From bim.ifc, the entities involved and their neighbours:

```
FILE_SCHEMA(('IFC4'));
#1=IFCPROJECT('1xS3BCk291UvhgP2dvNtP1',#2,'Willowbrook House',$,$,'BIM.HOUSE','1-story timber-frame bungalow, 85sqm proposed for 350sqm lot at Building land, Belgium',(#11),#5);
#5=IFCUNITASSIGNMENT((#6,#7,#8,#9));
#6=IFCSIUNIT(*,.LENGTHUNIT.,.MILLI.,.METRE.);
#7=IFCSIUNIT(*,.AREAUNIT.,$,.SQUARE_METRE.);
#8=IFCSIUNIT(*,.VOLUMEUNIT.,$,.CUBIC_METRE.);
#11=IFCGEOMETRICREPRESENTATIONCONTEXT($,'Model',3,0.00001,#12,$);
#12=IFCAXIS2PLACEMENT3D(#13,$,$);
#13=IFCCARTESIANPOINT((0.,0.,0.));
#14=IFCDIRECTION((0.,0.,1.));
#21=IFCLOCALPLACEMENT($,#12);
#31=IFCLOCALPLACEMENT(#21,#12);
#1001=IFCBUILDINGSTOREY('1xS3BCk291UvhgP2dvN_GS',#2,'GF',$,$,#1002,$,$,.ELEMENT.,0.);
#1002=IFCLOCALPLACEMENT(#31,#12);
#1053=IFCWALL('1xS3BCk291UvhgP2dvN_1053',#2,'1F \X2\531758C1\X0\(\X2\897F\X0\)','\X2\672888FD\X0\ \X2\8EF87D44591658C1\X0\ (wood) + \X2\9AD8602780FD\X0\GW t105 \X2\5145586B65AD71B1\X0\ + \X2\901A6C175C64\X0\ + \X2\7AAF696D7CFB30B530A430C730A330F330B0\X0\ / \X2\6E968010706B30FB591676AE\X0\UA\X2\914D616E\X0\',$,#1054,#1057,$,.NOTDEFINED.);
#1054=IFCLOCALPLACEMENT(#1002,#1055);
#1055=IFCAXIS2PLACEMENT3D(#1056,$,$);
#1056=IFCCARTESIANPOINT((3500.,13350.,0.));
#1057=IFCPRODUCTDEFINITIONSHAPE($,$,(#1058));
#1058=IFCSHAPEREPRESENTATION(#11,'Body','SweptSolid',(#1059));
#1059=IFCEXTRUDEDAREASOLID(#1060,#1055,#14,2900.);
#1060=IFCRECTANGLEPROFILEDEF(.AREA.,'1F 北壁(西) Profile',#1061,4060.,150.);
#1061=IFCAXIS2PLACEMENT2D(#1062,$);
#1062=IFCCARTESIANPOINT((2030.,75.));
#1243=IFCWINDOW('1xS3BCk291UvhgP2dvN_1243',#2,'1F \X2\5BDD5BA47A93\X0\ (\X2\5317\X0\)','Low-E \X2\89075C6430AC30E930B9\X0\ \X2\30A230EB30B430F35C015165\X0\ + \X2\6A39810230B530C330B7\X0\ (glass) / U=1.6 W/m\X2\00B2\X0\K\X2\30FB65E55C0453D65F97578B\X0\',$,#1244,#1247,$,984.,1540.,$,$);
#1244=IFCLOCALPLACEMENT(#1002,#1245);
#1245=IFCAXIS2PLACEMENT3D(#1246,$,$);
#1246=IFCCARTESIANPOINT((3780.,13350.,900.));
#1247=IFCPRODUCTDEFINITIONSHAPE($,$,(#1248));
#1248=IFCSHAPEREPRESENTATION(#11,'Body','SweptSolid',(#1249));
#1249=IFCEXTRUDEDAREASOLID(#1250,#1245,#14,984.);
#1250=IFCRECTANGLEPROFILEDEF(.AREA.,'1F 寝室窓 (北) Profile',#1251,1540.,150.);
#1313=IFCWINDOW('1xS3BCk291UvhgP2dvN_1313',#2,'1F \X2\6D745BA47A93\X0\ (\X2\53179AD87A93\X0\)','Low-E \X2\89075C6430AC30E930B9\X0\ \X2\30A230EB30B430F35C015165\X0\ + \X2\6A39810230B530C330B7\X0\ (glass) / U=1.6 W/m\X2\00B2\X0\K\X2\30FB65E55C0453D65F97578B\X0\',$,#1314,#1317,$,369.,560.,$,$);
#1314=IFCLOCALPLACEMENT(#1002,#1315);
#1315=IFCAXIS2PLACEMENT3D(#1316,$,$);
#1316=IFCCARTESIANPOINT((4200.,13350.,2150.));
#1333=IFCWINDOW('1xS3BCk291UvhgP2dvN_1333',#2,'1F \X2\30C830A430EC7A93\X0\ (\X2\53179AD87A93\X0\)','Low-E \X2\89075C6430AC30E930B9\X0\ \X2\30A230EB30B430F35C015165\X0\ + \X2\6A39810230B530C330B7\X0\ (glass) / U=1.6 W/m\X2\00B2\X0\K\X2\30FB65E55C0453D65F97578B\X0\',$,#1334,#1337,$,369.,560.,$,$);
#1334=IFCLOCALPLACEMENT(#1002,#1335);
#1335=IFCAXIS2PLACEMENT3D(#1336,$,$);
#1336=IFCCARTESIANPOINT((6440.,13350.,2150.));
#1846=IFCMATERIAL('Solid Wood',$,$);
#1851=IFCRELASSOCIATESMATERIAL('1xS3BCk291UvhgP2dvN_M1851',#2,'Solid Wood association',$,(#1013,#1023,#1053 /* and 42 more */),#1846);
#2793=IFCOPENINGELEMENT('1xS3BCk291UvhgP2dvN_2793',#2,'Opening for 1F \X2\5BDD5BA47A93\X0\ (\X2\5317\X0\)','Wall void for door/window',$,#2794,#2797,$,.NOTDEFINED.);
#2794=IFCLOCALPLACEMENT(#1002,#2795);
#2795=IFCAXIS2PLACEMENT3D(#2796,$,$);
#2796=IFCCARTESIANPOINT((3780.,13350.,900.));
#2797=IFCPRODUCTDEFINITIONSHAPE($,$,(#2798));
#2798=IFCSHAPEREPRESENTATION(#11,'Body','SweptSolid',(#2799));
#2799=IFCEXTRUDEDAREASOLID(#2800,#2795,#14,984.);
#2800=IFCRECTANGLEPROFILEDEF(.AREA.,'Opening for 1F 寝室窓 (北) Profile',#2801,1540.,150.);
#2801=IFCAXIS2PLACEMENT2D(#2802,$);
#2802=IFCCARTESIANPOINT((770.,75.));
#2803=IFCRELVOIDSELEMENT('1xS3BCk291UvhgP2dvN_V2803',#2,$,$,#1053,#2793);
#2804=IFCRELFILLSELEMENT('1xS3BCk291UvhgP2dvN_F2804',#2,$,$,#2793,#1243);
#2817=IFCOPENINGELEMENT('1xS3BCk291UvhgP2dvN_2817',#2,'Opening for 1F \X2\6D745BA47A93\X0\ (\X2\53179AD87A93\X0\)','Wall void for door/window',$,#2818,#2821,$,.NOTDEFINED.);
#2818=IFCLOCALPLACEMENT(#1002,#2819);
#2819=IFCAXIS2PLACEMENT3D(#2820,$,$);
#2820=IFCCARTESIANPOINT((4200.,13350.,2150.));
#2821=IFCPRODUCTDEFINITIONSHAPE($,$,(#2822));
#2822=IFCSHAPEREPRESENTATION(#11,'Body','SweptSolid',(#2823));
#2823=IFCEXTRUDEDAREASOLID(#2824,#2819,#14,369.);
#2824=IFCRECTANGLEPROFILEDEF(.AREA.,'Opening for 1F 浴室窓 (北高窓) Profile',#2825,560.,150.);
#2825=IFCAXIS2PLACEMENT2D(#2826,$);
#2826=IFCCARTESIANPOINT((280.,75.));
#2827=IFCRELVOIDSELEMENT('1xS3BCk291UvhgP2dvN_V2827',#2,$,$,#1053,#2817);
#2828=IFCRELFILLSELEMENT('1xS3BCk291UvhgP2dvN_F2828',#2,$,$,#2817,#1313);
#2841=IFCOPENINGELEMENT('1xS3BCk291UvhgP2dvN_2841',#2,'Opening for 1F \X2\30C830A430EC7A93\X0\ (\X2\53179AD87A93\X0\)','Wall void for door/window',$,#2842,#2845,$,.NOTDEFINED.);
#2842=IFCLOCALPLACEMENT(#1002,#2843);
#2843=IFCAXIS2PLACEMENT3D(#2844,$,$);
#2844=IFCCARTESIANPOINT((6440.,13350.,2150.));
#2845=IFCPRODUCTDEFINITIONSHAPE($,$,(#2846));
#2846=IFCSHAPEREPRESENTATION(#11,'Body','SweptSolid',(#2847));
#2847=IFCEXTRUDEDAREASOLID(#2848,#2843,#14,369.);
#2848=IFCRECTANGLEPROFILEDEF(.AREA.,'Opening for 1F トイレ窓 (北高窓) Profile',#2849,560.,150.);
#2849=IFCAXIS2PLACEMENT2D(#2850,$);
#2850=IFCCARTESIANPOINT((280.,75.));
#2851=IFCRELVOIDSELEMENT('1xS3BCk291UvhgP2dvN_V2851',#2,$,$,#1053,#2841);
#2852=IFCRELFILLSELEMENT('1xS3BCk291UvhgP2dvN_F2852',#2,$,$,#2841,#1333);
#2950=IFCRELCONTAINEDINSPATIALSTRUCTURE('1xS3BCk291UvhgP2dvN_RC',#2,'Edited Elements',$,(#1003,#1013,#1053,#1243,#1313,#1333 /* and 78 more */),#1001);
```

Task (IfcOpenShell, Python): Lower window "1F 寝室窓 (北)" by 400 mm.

```python
import numpy as np
import ifcopenshell
import ifcopenshell.api.geometry
import ifcopenshell.util.placement
import ifcopenshell.util.unit

model = ifcopenshell.open("bim.ifc")
unit_scale = ifcopenshell.util.unit.calculate_unit_scale(model)

window = model.by_id(1243)
opening = window.FillsVoids[0].RelatingOpeningElement
dz = -0.4 / unit_scale

shift = np.array([0.0, 0.0, dz])
# The window is not placed relative to its opening, so move both.
for product in (opening, window):
    matrix = ifcopenshell.util.placement.get_local_placement(product.ObjectPlacement)
    matrix[:3, 3] += shift
    ifcopenshell.api.geometry.edit_object_placement(model, product=product, matrix=matrix, is_si=False)

print(f"moved by {dz * unit_scale:+.3f} m")

model.write("bim_rev.ifc")
```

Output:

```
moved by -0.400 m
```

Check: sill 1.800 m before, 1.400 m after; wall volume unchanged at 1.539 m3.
